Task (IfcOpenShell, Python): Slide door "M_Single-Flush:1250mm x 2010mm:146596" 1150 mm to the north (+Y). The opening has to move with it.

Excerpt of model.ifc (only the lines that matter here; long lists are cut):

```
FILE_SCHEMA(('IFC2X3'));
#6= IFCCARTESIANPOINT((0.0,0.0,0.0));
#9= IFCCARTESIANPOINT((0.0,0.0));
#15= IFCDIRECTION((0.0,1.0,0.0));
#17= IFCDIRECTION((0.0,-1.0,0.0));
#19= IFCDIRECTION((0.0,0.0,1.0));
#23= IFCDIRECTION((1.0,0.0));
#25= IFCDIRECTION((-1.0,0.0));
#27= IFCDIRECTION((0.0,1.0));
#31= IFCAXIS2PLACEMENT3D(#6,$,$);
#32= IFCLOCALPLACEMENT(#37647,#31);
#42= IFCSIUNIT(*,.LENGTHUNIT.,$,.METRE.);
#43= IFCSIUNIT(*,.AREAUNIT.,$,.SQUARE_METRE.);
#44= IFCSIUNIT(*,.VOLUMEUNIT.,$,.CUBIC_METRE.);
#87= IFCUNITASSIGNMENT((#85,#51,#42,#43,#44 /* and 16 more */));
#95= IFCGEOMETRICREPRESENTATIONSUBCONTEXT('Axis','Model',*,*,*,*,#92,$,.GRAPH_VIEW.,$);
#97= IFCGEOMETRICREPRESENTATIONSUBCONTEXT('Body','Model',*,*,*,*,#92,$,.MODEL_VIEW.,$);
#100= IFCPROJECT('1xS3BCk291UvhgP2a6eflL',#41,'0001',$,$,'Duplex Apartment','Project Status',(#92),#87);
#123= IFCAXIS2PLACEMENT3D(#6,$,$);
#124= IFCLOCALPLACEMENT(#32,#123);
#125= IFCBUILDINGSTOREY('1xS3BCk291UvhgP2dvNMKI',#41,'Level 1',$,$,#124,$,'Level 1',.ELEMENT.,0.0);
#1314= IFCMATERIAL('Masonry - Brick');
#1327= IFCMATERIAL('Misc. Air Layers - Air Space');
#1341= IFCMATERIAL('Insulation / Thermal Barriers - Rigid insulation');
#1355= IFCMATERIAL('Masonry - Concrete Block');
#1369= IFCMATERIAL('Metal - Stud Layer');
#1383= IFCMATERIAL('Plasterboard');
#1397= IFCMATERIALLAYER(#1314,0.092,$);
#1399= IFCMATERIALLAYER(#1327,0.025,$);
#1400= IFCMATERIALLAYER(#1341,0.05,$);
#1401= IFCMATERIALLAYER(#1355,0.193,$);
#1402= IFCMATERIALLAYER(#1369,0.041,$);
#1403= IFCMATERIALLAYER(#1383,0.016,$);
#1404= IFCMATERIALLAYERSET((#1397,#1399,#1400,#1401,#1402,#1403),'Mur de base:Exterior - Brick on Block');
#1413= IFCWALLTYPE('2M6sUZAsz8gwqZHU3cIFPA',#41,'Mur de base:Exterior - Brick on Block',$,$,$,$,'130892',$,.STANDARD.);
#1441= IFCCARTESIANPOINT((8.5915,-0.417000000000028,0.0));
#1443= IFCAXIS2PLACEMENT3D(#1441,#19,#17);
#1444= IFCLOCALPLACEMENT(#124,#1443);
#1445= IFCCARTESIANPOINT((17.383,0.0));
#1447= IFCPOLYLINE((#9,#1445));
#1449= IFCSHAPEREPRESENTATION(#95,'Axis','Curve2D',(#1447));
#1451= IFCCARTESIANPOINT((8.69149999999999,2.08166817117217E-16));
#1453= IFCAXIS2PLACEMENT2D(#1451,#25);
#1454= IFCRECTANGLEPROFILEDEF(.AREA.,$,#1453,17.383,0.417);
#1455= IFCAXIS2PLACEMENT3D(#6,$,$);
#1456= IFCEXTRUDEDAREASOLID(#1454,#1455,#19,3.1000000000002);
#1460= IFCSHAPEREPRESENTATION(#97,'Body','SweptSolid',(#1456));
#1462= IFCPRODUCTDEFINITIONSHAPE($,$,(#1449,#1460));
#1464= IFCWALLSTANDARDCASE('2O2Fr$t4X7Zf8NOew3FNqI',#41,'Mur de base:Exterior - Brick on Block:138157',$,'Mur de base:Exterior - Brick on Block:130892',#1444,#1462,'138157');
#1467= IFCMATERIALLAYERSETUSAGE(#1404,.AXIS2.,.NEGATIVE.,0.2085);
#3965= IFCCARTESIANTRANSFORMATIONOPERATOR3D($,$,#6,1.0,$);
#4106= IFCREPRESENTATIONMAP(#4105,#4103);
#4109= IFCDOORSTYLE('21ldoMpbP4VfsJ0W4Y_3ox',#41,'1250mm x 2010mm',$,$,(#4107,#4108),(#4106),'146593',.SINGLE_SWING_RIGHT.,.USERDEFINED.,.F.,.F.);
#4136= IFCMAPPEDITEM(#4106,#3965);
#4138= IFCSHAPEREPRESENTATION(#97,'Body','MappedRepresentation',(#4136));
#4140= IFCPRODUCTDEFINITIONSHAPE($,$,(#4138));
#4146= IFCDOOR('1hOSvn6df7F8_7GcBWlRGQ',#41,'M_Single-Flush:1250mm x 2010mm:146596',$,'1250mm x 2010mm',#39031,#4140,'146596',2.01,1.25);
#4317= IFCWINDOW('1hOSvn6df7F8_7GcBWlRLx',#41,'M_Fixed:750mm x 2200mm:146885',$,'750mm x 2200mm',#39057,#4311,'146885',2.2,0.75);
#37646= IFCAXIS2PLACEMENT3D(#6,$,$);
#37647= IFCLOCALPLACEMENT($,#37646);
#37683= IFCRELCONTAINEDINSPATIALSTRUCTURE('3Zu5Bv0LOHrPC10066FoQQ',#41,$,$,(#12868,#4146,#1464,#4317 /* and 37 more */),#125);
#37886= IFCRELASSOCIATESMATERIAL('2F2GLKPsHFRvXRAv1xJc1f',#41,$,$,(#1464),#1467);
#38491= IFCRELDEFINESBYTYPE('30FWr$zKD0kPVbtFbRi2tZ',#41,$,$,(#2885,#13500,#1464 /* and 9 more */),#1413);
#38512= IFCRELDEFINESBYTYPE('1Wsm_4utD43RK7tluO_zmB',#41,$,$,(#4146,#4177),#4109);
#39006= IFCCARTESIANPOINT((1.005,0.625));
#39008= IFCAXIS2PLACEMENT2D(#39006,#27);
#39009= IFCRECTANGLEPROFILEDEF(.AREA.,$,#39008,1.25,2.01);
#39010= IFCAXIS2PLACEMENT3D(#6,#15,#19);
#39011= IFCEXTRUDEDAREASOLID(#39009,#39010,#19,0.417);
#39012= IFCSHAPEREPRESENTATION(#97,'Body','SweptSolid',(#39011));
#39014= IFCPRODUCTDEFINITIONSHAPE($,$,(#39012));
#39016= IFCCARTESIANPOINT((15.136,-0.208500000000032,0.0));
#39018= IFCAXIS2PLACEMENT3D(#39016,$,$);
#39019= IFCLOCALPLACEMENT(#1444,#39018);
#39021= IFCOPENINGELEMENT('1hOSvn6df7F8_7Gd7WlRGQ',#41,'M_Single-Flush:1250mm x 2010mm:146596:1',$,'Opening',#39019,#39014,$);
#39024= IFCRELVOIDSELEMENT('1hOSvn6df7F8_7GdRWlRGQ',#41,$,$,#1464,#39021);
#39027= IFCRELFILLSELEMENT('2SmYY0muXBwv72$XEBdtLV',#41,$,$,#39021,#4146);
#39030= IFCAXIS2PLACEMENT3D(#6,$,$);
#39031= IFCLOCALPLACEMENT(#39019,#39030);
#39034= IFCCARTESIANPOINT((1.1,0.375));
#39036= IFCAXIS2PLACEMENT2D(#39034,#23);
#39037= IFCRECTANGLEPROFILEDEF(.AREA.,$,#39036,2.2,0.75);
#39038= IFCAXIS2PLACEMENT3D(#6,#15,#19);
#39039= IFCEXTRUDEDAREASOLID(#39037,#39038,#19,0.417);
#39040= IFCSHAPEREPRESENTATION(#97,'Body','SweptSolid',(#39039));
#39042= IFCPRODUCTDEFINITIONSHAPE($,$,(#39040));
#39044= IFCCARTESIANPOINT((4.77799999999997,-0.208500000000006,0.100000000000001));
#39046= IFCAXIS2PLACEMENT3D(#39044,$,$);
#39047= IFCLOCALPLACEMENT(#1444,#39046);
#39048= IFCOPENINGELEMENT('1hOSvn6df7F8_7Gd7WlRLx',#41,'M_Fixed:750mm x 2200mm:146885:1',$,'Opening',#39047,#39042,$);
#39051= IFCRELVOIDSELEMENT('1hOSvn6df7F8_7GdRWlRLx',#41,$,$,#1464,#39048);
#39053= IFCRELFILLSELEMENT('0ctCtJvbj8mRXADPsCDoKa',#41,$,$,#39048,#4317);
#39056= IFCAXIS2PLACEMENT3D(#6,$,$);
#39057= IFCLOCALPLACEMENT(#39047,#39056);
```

```python
import ifcopenshell
import ifcopenshell.api.geometry
import ifcopenshell.util.placement
import ifcopenshell.util.unit

model = ifcopenshell.open("model.ifc")
unit_scale = ifcopenshell.util.unit.calculate_unit_scale(model)

door = model.by_guid("1hOSvn6df7F8_7GcBWlRGQ")
opening = door.FillsVoids[0].RelatingOpeningElement
wall = opening.VoidsElements[0].RelatingBuildingElement

wall_matrix = ifcopenshell.util.placement.get_local_placement(wall.ObjectPlacement)
shift = wall_matrix[:3, 0] * -1.15 / unit_scale
before = ifcopenshell.util.placement.get_local_placement(door.ObjectPlacement)[:3, 3].copy()

# The door is placed relative to its opening, so it follows when the opening moves.
matrix = ifcopenshell.util.placement.get_local_placement(opening.ObjectPlacement)
matrix[:3, 3] += shift
ifcopenshell.api.geometry.edit_object_placement(
    model, product=opening, matrix=matrix, is_si=False, should_transform_children=True
)

after = ifcopenshell.util.placement.get_local_placement(door.ObjectPlacement)[:3, 3]
print("door moved by", (after - before).round(3) + 0.0)

model.write("model-out.ifc")
```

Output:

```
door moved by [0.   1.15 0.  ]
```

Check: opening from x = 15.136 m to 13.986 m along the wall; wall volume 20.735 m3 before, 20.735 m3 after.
